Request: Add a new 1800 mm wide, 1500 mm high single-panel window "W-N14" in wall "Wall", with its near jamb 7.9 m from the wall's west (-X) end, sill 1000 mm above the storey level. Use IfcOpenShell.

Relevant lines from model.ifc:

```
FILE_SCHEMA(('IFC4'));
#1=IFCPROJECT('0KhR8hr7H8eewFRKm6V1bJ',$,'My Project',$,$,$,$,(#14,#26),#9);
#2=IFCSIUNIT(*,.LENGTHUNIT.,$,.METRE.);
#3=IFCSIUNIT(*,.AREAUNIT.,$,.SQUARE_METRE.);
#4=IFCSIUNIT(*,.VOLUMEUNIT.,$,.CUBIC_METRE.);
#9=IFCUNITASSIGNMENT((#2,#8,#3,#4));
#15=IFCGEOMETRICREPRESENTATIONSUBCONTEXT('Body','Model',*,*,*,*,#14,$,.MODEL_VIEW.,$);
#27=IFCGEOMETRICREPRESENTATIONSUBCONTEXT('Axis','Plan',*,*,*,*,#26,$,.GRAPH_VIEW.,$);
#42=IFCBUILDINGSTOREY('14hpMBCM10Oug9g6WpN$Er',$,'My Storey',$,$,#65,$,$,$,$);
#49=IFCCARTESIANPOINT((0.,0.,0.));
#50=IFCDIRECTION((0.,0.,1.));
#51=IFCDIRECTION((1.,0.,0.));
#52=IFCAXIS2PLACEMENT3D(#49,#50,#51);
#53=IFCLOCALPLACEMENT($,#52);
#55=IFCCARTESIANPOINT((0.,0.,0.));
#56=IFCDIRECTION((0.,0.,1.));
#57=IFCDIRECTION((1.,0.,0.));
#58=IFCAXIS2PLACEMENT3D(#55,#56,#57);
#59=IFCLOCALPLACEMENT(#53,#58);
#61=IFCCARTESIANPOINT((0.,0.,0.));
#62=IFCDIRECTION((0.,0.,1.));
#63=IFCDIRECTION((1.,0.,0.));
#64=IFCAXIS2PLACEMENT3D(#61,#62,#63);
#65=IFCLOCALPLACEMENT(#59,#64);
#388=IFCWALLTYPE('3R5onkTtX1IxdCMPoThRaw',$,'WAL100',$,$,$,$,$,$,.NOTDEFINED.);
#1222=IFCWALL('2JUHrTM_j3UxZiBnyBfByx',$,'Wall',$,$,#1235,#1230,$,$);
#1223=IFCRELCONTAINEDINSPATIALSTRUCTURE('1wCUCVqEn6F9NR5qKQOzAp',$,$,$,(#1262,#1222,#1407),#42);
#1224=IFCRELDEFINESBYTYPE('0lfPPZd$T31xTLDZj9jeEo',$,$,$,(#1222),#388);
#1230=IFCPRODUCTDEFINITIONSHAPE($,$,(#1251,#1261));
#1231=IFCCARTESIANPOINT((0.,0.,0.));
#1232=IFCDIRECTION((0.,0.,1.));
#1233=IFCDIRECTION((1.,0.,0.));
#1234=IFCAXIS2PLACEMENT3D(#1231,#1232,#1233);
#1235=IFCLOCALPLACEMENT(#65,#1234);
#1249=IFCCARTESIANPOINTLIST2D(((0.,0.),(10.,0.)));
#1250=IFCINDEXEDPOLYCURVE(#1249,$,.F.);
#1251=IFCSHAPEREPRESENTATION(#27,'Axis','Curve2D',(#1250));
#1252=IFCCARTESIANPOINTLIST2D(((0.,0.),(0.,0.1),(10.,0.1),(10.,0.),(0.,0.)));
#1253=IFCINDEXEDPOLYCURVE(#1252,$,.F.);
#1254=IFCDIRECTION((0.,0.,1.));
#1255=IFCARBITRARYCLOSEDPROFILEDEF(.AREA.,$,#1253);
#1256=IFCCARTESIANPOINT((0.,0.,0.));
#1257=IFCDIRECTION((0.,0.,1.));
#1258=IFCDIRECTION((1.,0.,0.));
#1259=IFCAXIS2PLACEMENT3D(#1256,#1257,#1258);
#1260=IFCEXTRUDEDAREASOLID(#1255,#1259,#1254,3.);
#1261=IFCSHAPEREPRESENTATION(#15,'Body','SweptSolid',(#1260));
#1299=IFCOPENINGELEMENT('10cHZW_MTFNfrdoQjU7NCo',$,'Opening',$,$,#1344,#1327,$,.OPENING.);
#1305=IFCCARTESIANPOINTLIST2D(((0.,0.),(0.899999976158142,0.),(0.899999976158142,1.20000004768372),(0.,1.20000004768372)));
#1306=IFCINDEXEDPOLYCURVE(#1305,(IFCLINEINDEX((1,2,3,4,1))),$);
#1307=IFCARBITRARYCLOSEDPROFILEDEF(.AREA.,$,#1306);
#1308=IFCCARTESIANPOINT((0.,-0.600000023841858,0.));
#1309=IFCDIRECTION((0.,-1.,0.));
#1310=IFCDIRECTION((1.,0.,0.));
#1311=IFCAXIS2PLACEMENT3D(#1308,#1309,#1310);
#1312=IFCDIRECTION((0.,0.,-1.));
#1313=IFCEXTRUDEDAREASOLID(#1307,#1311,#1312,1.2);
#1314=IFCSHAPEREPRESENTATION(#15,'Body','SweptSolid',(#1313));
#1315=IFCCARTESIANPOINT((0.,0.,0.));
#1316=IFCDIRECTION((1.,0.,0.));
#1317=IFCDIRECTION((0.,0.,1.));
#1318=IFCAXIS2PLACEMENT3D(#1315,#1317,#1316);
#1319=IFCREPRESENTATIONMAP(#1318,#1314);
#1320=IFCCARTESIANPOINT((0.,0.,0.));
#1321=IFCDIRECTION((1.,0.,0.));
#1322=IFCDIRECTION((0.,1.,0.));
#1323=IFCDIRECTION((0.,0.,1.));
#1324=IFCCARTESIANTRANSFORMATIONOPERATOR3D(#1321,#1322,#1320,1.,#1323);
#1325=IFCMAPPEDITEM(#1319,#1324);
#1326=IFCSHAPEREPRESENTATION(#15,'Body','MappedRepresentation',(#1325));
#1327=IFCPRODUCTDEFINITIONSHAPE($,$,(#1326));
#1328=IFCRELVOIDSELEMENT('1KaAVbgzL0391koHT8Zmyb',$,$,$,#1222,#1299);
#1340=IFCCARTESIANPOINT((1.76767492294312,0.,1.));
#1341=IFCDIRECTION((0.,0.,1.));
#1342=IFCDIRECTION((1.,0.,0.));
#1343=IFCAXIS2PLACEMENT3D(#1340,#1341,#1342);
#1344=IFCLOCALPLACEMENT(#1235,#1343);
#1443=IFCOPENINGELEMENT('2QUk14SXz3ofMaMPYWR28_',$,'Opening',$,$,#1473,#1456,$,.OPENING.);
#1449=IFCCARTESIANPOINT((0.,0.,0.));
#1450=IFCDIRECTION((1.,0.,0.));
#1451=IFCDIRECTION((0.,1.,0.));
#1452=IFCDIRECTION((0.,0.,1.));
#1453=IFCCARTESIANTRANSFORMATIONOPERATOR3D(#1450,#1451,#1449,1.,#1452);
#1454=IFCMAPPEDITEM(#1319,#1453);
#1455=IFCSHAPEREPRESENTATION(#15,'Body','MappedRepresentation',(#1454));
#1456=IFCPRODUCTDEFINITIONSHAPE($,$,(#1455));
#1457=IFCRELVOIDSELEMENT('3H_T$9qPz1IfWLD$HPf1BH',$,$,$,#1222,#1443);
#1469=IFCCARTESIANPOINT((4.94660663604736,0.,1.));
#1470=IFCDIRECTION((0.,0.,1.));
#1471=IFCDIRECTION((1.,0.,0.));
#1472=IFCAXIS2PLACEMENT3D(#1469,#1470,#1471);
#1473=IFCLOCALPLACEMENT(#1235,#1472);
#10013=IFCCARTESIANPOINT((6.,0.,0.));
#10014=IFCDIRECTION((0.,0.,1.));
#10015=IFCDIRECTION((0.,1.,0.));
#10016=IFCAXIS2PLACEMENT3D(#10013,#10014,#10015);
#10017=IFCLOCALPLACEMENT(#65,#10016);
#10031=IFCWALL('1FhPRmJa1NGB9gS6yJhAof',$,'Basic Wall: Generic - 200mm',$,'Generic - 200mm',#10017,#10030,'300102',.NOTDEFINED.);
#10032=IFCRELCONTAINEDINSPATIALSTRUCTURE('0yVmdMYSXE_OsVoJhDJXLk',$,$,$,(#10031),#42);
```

```python
import numpy as np
import ifcopenshell
import ifcopenshell.api.feature
import ifcopenshell.api.geometry
import ifcopenshell.api.root
import ifcopenshell.api.spatial
import ifcopenshell.geom
import ifcopenshell.util.element
import ifcopenshell.util.placement
import ifcopenshell.util.representation
import ifcopenshell.util.shape
import ifcopenshell.util.unit

model = ifcopenshell.open("model.ifc")
unit_scale = ifcopenshell.util.unit.calculate_unit_scale(model)
settings = ifcopenshell.geom.settings()


def volume(element):
    """Net volume in cubic metres, openings subtracted."""
    shape = ifcopenshell.geom.create_shape(settings, element)
    return ifcopenshell.util.shape.get_volume(shape.geometry)


wall = model.by_guid("2JUHrTM_j3UxZiBnyBfByx")
storey = ifcopenshell.util.element.get_container(wall, ifc_class="IfcBuildingStorey")
context = ifcopenshell.util.representation.get_context(model, "Model", "Body", "MODEL_VIEW")
before = volume(wall)

width, height, from_end, sill = 1.8, 1.5, 7.9, 1  # metres

# The wall runs along its own X axis, and the end named is its -X end.
wall_shape = ifcopenshell.geom.create_shape(settings, wall)
x, y, z = ifcopenshell.util.shape.get_vertices(wall_shape.geometry).T
start = x.min() + from_end
face, thickness = float(y.min()), float(y.max() - y.min())
wall_matrix = ifcopenshell.util.placement.get_local_placement(wall.ObjectPlacement)
level = ifcopenshell.util.placement.get_local_placement(storey.ObjectPlacement)[2, 3]


def in_wall(x, y):
    """Placement at x, y metres in the wall's axes, at sill height."""
    matrix = wall_matrix.copy()
    matrix[:, 3] = wall_matrix @ np.array([x / unit_scale, y / unit_scale, 0.0, 1.0])
    matrix[2, 3] = level + sill / unit_scale
    return matrix


# Opening: a box that overshoots both wall faces by 50 mm.
opening = ifcopenshell.api.root.create_entity(model, ifc_class="IfcOpeningElement", predefined_type="OPENING")
box = ifcopenshell.api.geometry.add_wall_representation(
    model, context=context, length=width, height=height, thickness=thickness + 0.1
)
ifcopenshell.api.geometry.assign_representation(model, product=opening, representation=box)
ifcopenshell.api.geometry.edit_object_placement(model, product=opening, matrix=in_wall(start, face - 0.05), is_si=False)
ifcopenshell.api.feature.add_feature(model, feature=opening, element=wall)

window = ifcopenshell.api.root.create_entity(model, ifc_class="IfcWindow", name="W-N14", predefined_type="WINDOW")
window.OverallWidth, window.OverallHeight = width / unit_scale, height / unit_scale
window.PartitioningType = "SINGLE_PANEL"
body = ifcopenshell.api.geometry.add_window_representation(
    model,
    context=context,
    overall_width=window.OverallWidth,
    overall_height=window.OverallHeight,
    partition_type="SINGLE_PANEL",
)
ifcopenshell.api.geometry.assign_representation(model, product=window, representation=body)
ifcopenshell.api.spatial.assign_container(model, products=[window], relating_structure=storey)
ifcopenshell.api.feature.add_filling(model, opening=opening, element=window)

# Centre the window in the wall's thickness.
ifcopenshell.api.geometry.edit_object_placement(model, product=window, matrix=in_wall(start, face), is_si=False)
window_shape = ifcopenshell.geom.create_shape(settings, window)
depth = ifcopenshell.util.shape.get_vertices(window_shape.geometry)[:, 1]
offset = face + thickness / 2 - (depth.min() + depth.max()) / 2
ifcopenshell.api.geometry.edit_object_placement(model, product=window, matrix=in_wall(start, offset), is_si=False)

after = volume(wall)

print(f"wall volume {before:.3f} -> {after:.3f} m3")

model.write("model_updated.ifc")
```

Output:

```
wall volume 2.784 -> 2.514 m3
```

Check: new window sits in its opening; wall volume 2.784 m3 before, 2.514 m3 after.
